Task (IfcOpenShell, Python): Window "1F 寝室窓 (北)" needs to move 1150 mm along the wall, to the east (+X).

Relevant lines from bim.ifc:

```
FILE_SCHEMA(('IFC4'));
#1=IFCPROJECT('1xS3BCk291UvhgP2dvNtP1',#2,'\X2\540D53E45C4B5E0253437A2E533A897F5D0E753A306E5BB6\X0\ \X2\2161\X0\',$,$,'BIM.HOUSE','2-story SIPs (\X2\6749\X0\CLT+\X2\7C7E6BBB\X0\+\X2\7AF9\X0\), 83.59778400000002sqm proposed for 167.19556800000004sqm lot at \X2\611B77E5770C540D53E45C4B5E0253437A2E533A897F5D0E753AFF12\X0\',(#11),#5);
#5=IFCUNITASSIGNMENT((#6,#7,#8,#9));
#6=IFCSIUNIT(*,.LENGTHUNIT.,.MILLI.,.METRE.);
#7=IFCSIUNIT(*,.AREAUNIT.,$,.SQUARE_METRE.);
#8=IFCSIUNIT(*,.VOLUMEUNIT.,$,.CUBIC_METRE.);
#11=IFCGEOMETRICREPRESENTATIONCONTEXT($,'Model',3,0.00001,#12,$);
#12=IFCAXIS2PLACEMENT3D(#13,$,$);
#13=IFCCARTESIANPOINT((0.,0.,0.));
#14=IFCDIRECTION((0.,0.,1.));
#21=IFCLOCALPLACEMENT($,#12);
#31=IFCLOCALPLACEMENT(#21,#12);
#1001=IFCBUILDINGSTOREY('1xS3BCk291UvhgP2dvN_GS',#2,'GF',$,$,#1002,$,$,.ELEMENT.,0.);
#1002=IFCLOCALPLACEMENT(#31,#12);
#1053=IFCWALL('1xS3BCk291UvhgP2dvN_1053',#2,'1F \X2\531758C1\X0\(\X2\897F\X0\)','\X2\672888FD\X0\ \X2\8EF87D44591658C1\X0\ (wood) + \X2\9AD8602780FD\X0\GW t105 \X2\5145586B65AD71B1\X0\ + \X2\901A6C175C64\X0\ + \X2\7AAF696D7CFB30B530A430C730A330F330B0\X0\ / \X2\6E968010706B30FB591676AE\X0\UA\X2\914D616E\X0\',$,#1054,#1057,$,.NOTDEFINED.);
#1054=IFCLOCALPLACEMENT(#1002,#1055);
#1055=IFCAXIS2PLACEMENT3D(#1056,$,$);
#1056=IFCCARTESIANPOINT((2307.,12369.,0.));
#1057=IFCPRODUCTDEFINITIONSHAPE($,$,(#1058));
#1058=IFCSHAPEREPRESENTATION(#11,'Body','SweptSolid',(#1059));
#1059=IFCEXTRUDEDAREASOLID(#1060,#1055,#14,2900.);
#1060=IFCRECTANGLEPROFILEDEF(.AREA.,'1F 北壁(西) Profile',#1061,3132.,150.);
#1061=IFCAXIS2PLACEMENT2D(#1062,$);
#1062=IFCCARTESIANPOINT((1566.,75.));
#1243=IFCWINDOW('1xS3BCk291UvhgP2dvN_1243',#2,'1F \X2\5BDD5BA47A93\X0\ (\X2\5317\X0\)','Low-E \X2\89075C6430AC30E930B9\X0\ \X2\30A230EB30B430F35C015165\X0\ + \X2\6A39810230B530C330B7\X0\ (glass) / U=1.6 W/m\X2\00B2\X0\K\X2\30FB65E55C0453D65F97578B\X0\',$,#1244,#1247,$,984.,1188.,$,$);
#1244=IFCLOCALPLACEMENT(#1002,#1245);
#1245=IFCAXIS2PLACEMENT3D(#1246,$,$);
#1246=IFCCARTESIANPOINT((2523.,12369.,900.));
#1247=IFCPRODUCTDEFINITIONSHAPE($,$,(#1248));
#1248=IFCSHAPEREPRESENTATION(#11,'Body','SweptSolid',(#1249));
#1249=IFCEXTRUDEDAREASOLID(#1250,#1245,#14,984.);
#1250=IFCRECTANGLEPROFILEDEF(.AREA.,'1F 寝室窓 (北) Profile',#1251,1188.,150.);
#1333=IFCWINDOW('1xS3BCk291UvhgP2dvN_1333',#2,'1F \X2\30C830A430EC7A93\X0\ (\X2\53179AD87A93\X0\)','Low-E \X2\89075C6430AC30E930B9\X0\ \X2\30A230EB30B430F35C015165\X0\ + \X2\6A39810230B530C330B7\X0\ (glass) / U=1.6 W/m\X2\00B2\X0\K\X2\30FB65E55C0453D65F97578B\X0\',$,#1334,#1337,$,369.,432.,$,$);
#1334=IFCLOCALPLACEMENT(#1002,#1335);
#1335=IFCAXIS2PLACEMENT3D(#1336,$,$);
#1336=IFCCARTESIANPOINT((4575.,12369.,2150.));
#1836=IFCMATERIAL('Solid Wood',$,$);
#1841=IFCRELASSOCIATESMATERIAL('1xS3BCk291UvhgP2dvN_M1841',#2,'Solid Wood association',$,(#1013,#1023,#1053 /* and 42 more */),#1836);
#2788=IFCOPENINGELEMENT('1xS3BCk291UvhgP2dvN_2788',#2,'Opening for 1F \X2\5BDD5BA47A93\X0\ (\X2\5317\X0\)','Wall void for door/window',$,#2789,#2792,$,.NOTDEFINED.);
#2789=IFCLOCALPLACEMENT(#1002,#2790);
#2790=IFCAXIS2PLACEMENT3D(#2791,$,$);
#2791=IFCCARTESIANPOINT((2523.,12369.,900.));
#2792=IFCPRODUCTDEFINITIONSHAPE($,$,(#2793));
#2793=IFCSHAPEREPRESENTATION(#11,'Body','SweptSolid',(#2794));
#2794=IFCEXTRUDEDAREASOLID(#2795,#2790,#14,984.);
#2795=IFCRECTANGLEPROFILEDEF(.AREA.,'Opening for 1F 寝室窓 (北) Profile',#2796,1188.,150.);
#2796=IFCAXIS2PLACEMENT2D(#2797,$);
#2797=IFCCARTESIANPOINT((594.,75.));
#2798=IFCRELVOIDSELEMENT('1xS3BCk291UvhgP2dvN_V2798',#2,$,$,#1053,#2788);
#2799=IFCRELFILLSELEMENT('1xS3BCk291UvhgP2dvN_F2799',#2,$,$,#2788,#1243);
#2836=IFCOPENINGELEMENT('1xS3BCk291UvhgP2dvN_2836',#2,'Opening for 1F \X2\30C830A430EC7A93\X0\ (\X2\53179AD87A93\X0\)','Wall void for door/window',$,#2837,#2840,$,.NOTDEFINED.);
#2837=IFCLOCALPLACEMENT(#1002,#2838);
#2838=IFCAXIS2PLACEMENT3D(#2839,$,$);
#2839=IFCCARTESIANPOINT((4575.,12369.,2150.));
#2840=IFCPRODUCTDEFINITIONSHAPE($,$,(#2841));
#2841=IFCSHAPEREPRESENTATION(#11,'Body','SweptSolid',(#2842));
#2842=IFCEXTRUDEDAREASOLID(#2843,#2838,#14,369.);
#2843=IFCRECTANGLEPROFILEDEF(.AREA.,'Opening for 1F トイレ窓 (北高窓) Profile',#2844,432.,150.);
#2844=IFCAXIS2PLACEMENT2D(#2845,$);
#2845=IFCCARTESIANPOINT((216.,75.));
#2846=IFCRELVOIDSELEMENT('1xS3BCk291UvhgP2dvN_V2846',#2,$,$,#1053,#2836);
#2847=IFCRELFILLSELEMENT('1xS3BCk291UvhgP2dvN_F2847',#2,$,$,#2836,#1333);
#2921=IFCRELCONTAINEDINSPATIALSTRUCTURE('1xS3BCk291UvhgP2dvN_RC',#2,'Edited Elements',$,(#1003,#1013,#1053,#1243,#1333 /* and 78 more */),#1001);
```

```python
import ifcopenshell
import ifcopenshell.api.geometry
import ifcopenshell.util.placement

model = ifcopenshell.open("bim.ifc")

window = model.by_id(1243)
opening = window.FillsVoids[0].RelatingOpeningElement
wall = opening.VoidsElements[0].RelatingBuildingElement

wall_matrix = ifcopenshell.util.placement.get_local_placement(wall.ObjectPlacement)
shift = wall_matrix[:3, 0] * 1150.0
before = ifcopenshell.util.placement.get_local_placement(window.ObjectPlacement)[:3, 3].copy()

# The window is not placed relative to its opening, so move both.
for product in (opening, window):
    matrix = ifcopenshell.util.placement.get_local_placement(product.ObjectPlacement)
    matrix[:3, 3] += shift
    ifcopenshell.api.geometry.edit_object_placement(model, product=product, matrix=matrix, is_si=False)

after = ifcopenshell.util.placement.get_local_placement(window.ObjectPlacement)[:3, 3]
print("window moved by", (after - before).round(3) + 0.0)

model.write("bim_v2.ifc")
```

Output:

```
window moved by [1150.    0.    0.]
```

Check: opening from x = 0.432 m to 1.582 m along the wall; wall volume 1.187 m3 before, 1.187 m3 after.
